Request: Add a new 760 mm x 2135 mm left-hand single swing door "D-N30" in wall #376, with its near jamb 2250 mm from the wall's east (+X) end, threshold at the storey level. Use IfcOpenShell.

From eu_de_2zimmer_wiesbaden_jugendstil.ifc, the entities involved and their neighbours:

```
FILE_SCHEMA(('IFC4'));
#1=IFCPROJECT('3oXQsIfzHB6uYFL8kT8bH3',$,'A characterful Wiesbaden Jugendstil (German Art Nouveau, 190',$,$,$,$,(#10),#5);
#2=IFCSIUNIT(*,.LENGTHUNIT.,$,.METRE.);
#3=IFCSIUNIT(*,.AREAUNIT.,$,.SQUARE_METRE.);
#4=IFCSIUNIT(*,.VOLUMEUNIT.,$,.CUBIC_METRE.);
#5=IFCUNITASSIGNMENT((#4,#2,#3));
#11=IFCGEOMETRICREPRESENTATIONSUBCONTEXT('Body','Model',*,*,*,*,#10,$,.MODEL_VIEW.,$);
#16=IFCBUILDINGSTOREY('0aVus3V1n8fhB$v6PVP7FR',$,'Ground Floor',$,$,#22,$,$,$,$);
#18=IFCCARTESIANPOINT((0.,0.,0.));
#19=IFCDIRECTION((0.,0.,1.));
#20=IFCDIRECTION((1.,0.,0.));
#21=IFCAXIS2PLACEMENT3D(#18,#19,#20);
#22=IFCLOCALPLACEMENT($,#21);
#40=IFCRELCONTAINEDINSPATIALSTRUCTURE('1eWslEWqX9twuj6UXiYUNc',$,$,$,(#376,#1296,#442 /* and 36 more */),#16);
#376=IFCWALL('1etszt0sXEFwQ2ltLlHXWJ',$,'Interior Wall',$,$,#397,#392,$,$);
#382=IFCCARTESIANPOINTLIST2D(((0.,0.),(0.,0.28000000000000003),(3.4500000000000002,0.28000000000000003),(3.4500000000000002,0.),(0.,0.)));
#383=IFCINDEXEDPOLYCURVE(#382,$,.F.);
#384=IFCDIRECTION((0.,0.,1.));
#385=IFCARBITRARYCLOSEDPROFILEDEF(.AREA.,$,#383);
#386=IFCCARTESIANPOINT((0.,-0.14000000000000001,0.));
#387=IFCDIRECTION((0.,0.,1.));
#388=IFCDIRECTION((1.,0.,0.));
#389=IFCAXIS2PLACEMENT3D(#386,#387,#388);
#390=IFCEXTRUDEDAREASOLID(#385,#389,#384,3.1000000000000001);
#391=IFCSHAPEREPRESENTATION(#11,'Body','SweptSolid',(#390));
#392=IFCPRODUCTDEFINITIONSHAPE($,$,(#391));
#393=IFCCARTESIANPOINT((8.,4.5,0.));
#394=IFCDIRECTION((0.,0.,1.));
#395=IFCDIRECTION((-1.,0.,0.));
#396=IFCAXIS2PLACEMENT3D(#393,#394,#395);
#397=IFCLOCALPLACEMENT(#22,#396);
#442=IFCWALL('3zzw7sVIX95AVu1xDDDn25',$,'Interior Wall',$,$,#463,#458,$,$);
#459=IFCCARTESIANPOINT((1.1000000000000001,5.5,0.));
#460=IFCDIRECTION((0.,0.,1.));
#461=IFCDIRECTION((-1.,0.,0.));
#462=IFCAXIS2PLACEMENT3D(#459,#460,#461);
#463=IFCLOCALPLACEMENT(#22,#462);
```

```python
import numpy as np
import ifcopenshell
import ifcopenshell.api.feature
import ifcopenshell.api.geometry
import ifcopenshell.api.root
import ifcopenshell.api.spatial
import ifcopenshell.geom
import ifcopenshell.util.element
import ifcopenshell.util.placement
import ifcopenshell.util.representation
import ifcopenshell.util.shape
import ifcopenshell.util.unit

model = ifcopenshell.open("eu_de_2zimmer_wiesbaden_jugendstil.ifc")
unit_scale = ifcopenshell.util.unit.calculate_unit_scale(model)
settings = ifcopenshell.geom.settings()


def volume(element):
    """Net volume in cubic metres, openings subtracted."""
    shape = ifcopenshell.geom.create_shape(settings, element)
    return ifcopenshell.util.shape.get_volume(shape.geometry)


wall = model.by_guid("1etszt0sXEFwQ2ltLlHXWJ")
storey = ifcopenshell.util.element.get_container(wall, ifc_class="IfcBuildingStorey")
context = ifcopenshell.util.representation.get_context(model, "Model", "Body", "MODEL_VIEW")
before = volume(wall)

width, height, from_end, sill = 0.76, 2.135, 2.25, 0.0  # metres

# The wall runs along its own X axis, and the end named is its -X end.
wall_shape = ifcopenshell.geom.create_shape(settings, wall)
x, y, z = ifcopenshell.util.shape.get_vertices(wall_shape.geometry).T
start = x.min() + from_end
face, thickness = float(y.min()), float(y.max() - y.min())
wall_matrix = ifcopenshell.util.placement.get_local_placement(wall.ObjectPlacement)
level = ifcopenshell.util.placement.get_local_placement(storey.ObjectPlacement)[2, 3]


def in_wall(x, y):
    """Placement at x, y metres in the wall's axes, at sill height."""
    matrix = wall_matrix.copy()
    matrix[:, 3] = wall_matrix @ np.array([x / unit_scale, y / unit_scale, 0.0, 1.0])
    matrix[2, 3] = level + sill / unit_scale
    return matrix


# Opening: a box that overshoots both wall faces by 50 mm.
opening = ifcopenshell.api.root.create_entity(model, ifc_class="IfcOpeningElement", predefined_type="OPENING")
box = ifcopenshell.api.geometry.add_wall_representation(
    model, context=context, length=width, height=height, thickness=thickness + 0.1
)
ifcopenshell.api.geometry.assign_representation(model, product=opening, representation=box)
ifcopenshell.api.geometry.edit_object_placement(model, product=opening, matrix=in_wall(start, face - 0.05), is_si=False)
ifcopenshell.api.feature.add_feature(model, feature=opening, element=wall)

door = ifcopenshell.api.root.create_entity(model, ifc_class="IfcDoor", name="D-N30", predefined_type="DOOR")
door.OverallWidth, door.OverallHeight = width / unit_scale, height / unit_scale
door.OperationType = "SINGLE_SWING_LEFT"
body = ifcopenshell.api.geometry.add_door_representation(
    model,
    context=context,
    overall_width=door.OverallWidth,
    overall_height=door.OverallHeight,
    operation_type="SINGLE_SWING_LEFT",
    lining_properties={"LiningDepth": thickness / unit_scale, "ThresholdDepth": thickness / unit_scale},
)
ifcopenshell.api.geometry.assign_representation(model, product=door, representation=body)
ifcopenshell.api.spatial.assign_container(model, products=[door], relating_structure=storey)
ifcopenshell.api.feature.add_filling(model, opening=opening, element=door)

# The lining spans the wall, so the door starts at the wall face.
ifcopenshell.api.geometry.edit_object_placement(model, product=door, matrix=in_wall(start, face), is_si=False)

after = volume(wall)

print(f"wall volume {before:.3f} -> {after:.3f} m3")

model.write("eu_de_2zimmer_wiesbaden_jugendstil_rev.ifc")
```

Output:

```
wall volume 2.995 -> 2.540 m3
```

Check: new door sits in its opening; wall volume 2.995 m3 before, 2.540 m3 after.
